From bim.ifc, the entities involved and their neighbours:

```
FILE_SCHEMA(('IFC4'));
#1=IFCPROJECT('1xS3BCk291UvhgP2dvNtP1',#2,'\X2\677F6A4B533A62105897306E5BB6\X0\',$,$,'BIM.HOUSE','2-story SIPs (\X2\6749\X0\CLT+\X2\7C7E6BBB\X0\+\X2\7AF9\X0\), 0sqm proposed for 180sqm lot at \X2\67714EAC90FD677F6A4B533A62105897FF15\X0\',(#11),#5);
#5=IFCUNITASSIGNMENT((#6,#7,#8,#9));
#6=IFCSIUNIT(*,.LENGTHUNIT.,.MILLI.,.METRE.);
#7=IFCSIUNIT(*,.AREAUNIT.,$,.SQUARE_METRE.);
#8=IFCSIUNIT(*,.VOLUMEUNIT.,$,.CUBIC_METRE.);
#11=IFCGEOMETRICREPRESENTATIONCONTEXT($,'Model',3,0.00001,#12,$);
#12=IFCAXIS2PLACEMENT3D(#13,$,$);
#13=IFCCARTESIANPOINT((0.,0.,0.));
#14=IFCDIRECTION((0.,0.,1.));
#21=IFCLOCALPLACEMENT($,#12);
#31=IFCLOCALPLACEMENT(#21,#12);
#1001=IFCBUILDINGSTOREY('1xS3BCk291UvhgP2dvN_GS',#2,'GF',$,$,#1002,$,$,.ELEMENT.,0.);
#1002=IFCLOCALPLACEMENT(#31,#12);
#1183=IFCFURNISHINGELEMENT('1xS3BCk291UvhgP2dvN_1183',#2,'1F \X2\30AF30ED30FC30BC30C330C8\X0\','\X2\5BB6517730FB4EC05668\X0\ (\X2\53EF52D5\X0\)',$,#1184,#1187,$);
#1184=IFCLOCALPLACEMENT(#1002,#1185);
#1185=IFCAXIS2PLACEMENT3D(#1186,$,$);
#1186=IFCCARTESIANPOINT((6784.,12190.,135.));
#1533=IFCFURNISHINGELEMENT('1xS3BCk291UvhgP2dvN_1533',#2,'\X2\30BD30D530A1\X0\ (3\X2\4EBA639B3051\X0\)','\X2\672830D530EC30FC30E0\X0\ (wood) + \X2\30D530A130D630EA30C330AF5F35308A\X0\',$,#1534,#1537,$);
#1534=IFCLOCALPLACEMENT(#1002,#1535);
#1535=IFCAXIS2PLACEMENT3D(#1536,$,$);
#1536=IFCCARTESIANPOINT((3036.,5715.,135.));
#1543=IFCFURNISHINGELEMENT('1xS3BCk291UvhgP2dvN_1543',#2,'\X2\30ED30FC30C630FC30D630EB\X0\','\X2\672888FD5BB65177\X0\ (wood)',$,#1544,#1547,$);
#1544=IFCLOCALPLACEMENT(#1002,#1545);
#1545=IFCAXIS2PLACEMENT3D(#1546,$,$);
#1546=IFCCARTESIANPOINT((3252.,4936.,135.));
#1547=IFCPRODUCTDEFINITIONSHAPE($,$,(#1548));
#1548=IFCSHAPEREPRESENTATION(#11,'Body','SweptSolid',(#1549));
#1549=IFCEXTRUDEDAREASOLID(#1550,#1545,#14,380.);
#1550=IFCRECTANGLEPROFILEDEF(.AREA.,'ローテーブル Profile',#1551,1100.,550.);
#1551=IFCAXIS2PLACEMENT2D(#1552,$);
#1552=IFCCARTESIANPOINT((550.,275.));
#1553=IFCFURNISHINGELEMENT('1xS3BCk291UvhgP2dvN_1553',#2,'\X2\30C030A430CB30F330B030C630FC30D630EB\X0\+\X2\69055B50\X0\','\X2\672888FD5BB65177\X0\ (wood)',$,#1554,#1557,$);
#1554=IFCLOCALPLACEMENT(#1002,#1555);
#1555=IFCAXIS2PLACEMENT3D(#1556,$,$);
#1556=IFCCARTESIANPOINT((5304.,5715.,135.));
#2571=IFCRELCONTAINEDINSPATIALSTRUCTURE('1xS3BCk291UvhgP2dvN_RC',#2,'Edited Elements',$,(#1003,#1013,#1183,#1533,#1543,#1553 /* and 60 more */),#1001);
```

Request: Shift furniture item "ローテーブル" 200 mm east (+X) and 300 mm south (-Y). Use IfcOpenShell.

```python
import ifcopenshell
import ifcopenshell.api.geometry
import ifcopenshell.util.placement

model = ifcopenshell.open("bim.ifc")

item = model.by_id(1543)
matrix = ifcopenshell.util.placement.get_local_placement(item.ObjectPlacement)
matrix[0, 3] += 200.0
matrix[1, 3] -= 300.0
ifcopenshell.api.geometry.edit_object_placement(model, product=item, matrix=matrix, is_si=False)

print(ifcopenshell.util.placement.get_local_placement(item.ObjectPlacement).round(3) + 0.0)

model.write("bim_updated.ifc")
```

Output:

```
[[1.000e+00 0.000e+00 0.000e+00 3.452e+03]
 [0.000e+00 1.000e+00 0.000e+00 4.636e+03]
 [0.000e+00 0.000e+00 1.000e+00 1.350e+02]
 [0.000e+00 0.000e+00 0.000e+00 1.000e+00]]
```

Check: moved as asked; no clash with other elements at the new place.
